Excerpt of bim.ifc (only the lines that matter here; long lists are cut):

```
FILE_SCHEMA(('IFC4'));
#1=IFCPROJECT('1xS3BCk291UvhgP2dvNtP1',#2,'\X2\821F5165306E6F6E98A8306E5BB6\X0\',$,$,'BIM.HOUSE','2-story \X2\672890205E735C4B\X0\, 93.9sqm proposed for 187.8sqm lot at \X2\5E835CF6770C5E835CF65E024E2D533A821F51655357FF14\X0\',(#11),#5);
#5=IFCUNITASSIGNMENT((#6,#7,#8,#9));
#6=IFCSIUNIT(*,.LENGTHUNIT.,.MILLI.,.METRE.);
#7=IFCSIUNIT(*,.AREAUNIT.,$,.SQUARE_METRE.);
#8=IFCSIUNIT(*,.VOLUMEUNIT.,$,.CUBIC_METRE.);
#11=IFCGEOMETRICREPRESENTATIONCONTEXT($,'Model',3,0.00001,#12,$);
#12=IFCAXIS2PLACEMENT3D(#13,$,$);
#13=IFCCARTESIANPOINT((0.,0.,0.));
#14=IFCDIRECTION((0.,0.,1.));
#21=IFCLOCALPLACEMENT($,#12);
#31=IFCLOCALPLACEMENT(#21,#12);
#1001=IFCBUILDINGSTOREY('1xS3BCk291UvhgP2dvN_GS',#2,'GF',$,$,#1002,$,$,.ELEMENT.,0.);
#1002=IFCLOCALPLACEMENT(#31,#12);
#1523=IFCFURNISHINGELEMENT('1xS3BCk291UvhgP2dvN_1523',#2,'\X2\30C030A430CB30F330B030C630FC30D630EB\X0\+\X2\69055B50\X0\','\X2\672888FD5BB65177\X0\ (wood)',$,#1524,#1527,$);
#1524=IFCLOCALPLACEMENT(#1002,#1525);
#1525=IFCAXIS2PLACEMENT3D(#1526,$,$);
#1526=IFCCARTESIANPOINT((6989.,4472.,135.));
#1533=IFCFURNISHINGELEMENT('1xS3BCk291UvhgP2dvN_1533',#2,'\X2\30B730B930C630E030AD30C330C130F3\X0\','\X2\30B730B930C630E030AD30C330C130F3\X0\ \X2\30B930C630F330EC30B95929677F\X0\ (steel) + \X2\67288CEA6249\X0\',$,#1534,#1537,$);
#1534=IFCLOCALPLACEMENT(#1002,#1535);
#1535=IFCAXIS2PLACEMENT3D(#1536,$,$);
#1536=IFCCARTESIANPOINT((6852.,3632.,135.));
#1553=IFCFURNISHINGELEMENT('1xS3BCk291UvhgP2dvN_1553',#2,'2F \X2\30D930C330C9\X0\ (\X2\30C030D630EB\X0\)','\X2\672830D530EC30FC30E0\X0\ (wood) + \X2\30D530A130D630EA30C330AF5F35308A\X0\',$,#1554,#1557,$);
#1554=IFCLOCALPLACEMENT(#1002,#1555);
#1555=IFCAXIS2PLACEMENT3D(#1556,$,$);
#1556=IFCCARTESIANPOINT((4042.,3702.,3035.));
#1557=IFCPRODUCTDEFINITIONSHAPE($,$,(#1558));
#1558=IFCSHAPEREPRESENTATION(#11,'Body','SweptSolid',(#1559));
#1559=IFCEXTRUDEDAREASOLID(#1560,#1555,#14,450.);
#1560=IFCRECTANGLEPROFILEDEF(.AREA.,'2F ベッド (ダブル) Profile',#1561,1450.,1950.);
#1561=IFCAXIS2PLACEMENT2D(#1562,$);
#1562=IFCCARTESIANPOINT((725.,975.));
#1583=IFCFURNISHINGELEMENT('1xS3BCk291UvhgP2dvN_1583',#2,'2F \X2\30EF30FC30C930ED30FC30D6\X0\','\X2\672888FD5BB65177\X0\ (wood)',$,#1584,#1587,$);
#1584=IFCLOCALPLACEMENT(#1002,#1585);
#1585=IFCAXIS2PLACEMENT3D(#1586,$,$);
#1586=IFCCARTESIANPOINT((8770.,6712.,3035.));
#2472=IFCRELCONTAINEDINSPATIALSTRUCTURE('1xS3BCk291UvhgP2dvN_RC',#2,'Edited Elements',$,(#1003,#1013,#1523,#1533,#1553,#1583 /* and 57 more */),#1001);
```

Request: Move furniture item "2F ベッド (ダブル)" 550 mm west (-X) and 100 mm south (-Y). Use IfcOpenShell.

```python
import ifcopenshell
import ifcopenshell.api.geometry
import ifcopenshell.util.placement

model = ifcopenshell.open("bim.ifc")

item = model.by_guid("1xS3BCk291UvhgP2dvN_1553")
matrix = ifcopenshell.util.placement.get_local_placement(item.ObjectPlacement)
matrix[0, 3] -= 550.0
matrix[1, 3] -= 100.0
ifcopenshell.api.geometry.edit_object_placement(model, product=item, matrix=matrix, is_si=False)

print(ifcopenshell.util.placement.get_local_placement(item.ObjectPlacement).round(3) + 0.0)

model.write("bim_v2.ifc")
```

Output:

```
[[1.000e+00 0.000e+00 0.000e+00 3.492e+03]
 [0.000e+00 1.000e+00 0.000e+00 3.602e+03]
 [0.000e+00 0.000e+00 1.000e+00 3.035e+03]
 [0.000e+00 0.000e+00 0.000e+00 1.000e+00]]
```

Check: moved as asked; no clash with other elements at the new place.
